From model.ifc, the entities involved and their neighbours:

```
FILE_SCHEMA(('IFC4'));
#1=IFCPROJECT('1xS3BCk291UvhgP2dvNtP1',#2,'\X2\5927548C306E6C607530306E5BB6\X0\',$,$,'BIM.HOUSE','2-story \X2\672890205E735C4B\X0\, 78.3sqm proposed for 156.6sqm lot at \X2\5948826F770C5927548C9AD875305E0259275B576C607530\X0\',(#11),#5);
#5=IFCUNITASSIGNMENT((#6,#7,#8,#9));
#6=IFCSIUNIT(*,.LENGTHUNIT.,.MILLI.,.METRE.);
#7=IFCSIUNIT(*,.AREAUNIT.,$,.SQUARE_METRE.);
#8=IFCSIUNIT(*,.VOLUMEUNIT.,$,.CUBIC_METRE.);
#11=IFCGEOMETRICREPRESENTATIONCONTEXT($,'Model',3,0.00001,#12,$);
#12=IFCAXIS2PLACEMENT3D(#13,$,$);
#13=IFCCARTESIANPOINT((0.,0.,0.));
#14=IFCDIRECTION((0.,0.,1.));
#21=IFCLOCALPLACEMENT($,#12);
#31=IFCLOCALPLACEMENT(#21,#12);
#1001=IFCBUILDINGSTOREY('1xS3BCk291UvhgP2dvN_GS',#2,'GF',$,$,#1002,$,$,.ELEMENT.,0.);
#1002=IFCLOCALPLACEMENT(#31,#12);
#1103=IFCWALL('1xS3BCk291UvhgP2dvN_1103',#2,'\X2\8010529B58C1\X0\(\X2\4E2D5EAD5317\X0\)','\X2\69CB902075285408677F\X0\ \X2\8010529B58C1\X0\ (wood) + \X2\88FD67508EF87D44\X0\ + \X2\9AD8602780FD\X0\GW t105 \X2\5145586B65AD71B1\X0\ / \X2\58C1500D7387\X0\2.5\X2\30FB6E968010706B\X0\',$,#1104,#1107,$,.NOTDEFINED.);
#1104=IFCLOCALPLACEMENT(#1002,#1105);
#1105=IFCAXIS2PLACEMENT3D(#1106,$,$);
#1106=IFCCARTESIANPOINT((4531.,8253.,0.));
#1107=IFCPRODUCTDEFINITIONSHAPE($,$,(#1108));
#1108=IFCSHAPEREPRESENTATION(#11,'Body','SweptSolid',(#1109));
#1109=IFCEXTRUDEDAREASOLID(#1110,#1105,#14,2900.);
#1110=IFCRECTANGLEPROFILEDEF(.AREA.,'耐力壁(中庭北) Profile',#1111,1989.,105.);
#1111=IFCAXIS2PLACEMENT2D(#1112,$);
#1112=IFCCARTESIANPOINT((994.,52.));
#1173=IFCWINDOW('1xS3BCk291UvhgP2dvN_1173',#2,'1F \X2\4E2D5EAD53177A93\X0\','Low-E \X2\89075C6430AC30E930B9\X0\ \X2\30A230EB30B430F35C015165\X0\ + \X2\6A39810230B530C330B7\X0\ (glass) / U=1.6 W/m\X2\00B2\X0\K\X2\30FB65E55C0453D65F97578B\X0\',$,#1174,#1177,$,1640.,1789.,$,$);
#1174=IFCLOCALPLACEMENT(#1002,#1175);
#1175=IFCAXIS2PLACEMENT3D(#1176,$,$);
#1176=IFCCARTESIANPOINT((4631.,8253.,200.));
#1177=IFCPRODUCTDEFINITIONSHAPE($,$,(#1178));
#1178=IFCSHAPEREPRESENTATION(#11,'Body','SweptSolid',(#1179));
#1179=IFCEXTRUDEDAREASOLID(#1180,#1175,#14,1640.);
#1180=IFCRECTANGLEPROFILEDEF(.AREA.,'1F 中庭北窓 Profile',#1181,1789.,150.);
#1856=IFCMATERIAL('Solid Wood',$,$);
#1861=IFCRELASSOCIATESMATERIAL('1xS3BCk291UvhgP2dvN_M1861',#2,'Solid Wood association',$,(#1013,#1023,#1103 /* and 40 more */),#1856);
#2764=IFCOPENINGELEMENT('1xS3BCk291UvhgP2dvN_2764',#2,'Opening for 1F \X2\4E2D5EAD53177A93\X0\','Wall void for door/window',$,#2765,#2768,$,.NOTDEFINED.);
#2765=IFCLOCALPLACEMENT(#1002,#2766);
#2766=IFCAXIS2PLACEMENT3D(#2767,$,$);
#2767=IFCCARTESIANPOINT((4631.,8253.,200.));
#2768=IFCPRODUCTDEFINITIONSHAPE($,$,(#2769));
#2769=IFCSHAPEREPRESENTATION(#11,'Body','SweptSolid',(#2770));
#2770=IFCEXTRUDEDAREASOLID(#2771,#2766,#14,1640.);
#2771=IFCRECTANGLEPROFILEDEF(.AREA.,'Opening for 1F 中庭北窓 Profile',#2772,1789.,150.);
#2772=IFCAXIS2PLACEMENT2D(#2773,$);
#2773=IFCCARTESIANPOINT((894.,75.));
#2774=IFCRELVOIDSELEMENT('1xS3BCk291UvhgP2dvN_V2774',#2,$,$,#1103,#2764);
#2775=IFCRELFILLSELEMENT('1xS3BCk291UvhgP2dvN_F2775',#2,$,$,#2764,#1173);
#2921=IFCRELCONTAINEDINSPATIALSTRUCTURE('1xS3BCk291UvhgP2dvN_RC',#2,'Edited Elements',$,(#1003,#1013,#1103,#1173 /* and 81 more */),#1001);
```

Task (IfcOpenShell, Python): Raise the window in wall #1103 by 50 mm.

```python
import numpy as np
import ifcopenshell
import ifcopenshell.api.geometry
import ifcopenshell.util.placement
import ifcopenshell.util.unit

model = ifcopenshell.open("model.ifc")
unit_scale = ifcopenshell.util.unit.calculate_unit_scale(model)

window = model.by_guid("1xS3BCk291UvhgP2dvN_1173")
opening = window.FillsVoids[0].RelatingOpeningElement
dz = 50.0

shift = np.array([0.0, 0.0, dz])
# The window is not placed relative to its opening, so move both.
for product in (opening, window):
    matrix = ifcopenshell.util.placement.get_local_placement(product.ObjectPlacement)
    matrix[:3, 3] += shift
    ifcopenshell.api.geometry.edit_object_placement(model, product=product, matrix=matrix, is_si=False)

print(f"moved by {dz * unit_scale:+.3f} m")

model.write("model_v2.ifc")
```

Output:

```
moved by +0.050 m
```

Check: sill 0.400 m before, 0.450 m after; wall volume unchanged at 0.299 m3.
